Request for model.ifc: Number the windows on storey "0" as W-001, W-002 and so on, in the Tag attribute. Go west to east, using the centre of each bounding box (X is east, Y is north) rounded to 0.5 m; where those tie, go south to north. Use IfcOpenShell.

First a look at what the model holds.

```python
import ifcopenshell
import ifcopenshell.util.element
import ifcopenshell.util.placement

model = ifcopenshell.open("model.ifc")
print(model.schema)
storey = next(s for s in model.by_type("IfcBuildingStorey") if s.Name == "0")
windows = [e for e in ifcopenshell.util.element.get_decomposition(storey) if e.is_a("IfcWindow")]
for e in sorted(windows, key=lambda e: e.id()):
    origin = ifcopenshell.util.placement.get_local_placement(e.ObjectPlacement)[:3, 3]
    print(e.id(), e.Tag, e.Name, origin.round(2) + 0.0, sep=" | ")
```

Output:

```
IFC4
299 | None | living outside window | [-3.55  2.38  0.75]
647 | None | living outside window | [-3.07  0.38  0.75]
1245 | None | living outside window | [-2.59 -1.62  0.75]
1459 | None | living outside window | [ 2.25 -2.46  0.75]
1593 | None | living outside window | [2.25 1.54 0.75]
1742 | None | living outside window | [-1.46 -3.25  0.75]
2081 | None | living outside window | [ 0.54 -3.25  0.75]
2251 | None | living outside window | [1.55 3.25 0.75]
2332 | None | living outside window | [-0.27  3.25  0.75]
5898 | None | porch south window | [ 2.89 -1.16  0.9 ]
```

```python
import ifcopenshell
import ifcopenshell.geom
import ifcopenshell.util.element
import ifcopenshell.util.shape

model = ifcopenshell.open("model.ifc")
settings = ifcopenshell.geom.settings()
settings.set("use-world-coords", True)


def centre(element):
    shape = ifcopenshell.geom.create_shape(settings, element)
    return ifcopenshell.util.shape.get_bbox_centroid(shape.geometry)


storey = next(s for s in model.by_type("IfcBuildingStorey") if s.Name == "0")
windows = [e for e in ifcopenshell.util.element.get_decomposition(storey) if e.is_a("IfcWindow")]

# Insertion points can sit at a corner or the storey origin, so sort by the geometry (in metres).
centres = {e: centre(e) for e in windows}
windows.sort(key=lambda e: (round(centres[e][0] / 0.5), centres[e][1]))

for i, e in enumerate(windows, start=1):
    number = f"W-0{i:02d}"
    e.Tag = number
    print(e.id(), number)

model.write("model_updated.ifc")
```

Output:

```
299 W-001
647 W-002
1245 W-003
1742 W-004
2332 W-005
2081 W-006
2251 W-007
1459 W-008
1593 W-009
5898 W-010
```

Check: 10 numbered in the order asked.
